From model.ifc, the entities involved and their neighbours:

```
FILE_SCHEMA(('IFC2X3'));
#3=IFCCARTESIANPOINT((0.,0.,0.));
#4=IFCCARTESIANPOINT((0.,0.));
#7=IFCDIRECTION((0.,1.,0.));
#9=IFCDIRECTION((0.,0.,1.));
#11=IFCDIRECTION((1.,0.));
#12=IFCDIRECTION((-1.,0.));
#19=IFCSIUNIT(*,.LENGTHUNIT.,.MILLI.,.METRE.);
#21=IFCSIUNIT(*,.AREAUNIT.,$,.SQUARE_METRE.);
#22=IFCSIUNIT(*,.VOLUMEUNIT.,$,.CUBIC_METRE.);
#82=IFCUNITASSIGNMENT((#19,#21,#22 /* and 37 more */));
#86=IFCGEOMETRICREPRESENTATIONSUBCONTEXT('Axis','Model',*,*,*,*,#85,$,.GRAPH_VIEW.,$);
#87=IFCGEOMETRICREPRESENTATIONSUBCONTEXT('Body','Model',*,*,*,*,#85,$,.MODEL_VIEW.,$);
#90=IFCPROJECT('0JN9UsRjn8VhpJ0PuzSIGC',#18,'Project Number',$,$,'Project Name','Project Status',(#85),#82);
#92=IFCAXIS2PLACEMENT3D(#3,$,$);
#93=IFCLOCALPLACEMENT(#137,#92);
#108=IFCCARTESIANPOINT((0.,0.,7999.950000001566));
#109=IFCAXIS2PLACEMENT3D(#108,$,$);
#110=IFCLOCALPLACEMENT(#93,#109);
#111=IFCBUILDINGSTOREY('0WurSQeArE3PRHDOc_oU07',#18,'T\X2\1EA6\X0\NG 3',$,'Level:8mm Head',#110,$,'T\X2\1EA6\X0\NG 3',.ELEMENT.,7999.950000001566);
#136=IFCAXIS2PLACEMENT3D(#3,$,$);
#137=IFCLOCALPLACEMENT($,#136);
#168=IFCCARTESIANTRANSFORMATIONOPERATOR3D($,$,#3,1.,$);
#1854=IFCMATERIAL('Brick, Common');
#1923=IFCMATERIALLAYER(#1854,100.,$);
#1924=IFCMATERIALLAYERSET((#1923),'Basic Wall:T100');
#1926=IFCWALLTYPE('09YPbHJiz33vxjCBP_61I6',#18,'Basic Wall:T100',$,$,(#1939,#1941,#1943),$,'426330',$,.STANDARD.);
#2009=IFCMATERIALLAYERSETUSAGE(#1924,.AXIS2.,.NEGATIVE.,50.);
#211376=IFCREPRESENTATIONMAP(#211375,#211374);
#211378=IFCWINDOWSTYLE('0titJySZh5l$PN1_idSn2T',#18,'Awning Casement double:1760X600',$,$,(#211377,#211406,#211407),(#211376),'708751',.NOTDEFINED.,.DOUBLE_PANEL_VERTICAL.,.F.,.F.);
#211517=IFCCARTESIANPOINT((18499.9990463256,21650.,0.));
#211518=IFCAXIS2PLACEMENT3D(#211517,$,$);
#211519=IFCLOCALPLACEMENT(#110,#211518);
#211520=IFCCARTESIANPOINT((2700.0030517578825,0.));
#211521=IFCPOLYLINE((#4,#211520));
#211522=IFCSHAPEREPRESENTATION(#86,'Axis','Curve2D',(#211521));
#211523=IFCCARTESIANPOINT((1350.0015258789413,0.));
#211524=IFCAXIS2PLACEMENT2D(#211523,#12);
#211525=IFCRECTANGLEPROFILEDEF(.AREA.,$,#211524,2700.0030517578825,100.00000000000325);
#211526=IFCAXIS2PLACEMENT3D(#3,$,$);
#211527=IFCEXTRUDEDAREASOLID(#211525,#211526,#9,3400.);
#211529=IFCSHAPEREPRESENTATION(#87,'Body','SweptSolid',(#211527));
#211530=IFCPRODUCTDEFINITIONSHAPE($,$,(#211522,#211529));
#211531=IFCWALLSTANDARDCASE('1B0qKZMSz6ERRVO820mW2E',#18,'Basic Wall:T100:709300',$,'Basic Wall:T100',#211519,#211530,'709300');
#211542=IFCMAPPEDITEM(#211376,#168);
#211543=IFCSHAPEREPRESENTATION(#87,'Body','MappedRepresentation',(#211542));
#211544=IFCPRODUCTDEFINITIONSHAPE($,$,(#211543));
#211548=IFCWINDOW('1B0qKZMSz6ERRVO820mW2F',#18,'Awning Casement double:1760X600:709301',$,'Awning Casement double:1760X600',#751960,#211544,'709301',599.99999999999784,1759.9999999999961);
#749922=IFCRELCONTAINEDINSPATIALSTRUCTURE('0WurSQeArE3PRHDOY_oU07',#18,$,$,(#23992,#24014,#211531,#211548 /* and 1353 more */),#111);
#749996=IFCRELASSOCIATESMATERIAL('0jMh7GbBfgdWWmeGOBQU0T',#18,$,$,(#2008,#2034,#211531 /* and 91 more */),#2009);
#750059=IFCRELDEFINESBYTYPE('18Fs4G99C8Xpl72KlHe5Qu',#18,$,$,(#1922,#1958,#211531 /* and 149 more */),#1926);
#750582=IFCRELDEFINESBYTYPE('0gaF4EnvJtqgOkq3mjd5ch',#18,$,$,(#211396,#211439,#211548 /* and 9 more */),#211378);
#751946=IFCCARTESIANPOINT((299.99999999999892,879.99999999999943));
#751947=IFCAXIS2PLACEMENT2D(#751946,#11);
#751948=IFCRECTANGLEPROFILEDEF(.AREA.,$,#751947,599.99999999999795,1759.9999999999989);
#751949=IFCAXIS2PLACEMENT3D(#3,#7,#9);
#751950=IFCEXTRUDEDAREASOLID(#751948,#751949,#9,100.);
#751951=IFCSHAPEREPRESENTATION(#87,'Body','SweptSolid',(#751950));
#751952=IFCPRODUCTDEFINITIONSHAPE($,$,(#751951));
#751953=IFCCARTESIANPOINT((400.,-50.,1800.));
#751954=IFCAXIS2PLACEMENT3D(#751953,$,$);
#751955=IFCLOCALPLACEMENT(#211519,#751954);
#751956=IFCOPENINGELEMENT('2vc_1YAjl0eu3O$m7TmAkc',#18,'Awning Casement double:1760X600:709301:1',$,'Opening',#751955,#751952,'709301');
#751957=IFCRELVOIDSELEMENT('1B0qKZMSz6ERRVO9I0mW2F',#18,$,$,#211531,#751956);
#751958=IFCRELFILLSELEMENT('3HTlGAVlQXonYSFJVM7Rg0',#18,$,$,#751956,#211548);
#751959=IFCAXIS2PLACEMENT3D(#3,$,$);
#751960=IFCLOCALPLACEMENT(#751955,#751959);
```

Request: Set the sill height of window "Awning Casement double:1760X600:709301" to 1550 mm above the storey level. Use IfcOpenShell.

```python
import numpy as np
import ifcopenshell
import ifcopenshell.api.geometry
import ifcopenshell.geom
import ifcopenshell.util.element
import ifcopenshell.util.placement
import ifcopenshell.util.shape
import ifcopenshell.util.unit

model = ifcopenshell.open("model.ifc")
unit_scale = ifcopenshell.util.unit.calculate_unit_scale(model)

window = model.by_guid("1B0qKZMSz6ERRVO820mW2F")
opening = window.FillsVoids[0].RelatingOpeningElement
storey = ifcopenshell.util.element.get_container(window, ifc_class="IfcBuildingStorey")
level = ifcopenshell.util.placement.get_local_placement(storey.ObjectPlacement)[2, 3]

# The opening's origin need not be at the sill, so measure its lowest point.
shape = ifcopenshell.geom.create_shape(ifcopenshell.geom.settings(), opening)
bottom = ifcopenshell.util.shape.get_shape_bottom_elevation(shape, shape.geometry) / unit_scale
dz = level + 1550.0 - bottom

shift = np.array([0.0, 0.0, dz])
# The window is placed relative to its opening, so it follows when the opening moves.
matrix = ifcopenshell.util.placement.get_local_placement(opening.ObjectPlacement)
matrix[:3, 3] += shift
ifcopenshell.api.geometry.edit_object_placement(
    model, product=opening, matrix=matrix, is_si=False, should_transform_children=True
)

print(f"moved by {dz * unit_scale:+.3f} m")

model.write("model_rev.ifc")
```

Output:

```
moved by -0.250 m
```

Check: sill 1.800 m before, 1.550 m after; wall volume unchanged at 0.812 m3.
